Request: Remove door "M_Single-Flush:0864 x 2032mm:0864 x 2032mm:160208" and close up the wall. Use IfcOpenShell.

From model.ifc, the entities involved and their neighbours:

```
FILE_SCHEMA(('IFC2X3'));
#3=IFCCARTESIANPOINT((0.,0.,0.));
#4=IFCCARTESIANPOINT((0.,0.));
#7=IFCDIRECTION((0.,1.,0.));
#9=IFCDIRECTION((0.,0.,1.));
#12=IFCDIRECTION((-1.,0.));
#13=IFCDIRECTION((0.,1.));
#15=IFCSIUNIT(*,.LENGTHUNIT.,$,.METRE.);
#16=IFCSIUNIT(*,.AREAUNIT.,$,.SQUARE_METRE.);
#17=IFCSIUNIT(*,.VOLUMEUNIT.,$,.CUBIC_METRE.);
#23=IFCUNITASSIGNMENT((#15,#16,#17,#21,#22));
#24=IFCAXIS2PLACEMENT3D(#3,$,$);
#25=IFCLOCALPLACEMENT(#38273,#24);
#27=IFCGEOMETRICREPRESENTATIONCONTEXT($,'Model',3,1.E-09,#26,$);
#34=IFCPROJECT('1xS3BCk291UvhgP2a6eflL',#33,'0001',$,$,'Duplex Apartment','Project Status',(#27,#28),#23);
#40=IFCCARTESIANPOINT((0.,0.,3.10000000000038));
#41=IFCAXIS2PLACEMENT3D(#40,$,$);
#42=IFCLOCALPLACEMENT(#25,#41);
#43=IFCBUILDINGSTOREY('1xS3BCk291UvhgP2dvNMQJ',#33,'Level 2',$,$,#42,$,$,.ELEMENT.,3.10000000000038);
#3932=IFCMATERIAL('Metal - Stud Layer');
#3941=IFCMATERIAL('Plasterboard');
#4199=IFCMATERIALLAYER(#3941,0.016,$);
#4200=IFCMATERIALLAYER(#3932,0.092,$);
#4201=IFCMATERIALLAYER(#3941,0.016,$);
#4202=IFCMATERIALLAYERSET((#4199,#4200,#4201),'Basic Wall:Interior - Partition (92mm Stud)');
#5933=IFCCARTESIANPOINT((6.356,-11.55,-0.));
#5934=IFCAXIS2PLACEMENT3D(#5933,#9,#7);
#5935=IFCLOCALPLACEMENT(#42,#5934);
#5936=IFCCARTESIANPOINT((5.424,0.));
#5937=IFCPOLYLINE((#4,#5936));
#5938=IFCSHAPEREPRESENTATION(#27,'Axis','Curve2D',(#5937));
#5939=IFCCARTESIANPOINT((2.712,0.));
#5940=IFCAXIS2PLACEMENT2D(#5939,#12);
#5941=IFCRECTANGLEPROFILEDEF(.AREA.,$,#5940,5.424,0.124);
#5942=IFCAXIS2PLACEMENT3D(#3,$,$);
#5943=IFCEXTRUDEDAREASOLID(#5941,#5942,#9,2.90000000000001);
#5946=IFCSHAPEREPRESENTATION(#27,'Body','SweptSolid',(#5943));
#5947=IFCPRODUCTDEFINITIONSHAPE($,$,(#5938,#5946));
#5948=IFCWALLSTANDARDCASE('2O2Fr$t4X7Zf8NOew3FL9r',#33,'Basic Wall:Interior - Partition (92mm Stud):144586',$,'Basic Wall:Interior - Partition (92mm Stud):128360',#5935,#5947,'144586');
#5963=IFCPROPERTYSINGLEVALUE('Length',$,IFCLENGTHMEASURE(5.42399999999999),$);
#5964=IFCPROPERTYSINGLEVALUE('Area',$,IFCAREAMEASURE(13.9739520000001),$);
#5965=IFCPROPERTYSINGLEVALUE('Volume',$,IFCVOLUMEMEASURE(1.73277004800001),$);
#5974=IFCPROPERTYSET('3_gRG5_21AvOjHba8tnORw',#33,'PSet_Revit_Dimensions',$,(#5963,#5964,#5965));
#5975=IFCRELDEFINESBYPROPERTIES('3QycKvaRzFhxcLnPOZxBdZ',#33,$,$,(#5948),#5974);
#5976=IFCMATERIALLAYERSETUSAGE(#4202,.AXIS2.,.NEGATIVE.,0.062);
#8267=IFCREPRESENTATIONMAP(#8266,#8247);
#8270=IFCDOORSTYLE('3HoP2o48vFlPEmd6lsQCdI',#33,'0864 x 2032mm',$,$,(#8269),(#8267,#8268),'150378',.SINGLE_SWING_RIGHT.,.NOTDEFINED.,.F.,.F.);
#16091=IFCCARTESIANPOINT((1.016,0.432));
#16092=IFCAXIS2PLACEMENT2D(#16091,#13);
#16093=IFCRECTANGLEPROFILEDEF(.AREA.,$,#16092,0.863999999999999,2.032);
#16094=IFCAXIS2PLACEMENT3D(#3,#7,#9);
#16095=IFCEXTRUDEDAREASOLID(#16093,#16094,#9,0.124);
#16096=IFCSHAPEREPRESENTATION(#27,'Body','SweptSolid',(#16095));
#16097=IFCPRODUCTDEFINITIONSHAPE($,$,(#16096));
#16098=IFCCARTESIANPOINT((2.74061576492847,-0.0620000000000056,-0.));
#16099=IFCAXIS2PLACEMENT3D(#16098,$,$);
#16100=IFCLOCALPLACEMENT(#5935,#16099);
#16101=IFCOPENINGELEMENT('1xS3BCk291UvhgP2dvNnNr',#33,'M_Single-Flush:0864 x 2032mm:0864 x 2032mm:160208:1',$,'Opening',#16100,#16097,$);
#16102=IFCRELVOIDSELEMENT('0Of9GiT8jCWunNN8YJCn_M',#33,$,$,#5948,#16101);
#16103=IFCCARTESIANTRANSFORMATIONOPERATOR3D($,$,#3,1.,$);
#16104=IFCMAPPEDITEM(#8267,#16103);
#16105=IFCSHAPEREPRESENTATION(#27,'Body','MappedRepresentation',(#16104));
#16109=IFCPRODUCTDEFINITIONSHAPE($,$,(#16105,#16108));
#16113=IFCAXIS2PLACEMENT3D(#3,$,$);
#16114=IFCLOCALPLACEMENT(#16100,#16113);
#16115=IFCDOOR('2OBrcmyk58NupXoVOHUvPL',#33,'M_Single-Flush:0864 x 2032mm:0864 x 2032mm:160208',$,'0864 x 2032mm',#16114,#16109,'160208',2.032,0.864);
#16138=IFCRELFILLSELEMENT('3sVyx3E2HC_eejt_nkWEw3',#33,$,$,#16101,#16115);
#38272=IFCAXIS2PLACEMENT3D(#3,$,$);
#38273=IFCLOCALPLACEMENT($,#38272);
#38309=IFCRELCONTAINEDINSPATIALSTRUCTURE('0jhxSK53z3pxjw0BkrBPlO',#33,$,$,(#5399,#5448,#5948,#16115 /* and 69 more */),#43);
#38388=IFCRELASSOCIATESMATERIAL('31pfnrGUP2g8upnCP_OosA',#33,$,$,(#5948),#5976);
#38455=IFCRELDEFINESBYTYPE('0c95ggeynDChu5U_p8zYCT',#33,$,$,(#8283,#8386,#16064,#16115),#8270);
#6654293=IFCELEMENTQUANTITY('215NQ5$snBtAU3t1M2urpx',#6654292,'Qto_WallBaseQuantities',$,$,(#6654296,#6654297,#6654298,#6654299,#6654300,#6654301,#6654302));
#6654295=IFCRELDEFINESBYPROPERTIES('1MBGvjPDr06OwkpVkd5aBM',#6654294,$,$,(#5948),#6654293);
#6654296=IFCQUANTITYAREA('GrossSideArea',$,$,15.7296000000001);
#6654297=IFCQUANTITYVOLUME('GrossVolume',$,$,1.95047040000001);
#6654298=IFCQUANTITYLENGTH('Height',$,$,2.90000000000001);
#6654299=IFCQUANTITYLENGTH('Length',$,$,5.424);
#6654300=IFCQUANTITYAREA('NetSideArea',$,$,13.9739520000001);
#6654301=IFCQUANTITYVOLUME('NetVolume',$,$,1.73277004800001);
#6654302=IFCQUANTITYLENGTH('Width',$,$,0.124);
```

```python
import ifcopenshell
import ifcopenshell.api.feature
import ifcopenshell.api.pset
import ifcopenshell.api.root
import ifcopenshell.geom
import ifcopenshell.util.element
import ifcopenshell.util.shape
import ifcopenshell.util.unit

model = ifcopenshell.open("model.ifc")
area_scale = ifcopenshell.util.unit.calculate_unit_scale(model, "AREAUNIT")
volume_scale = ifcopenshell.util.unit.calculate_unit_scale(model, "VOLUMEUNIT")
settings = ifcopenshell.geom.settings()


def volume(element):
    """Net volume in cubic metres, openings subtracted."""
    shape = ifcopenshell.geom.create_shape(settings, element)
    return ifcopenshell.util.shape.get_volume(shape.geometry)


door = model.by_guid("2OBrcmyk58NupXoVOHUvPL")
opening = door.FillsVoids[0].RelatingOpeningElement
wall = opening.VoidsElements[0].RelatingBuildingElement
before = volume(wall)

ifcopenshell.api.root.remove_product(model, product=door)
ifcopenshell.api.feature.remove_feature(model, feature=opening)

after = volume(wall)
thickness = 0.124  # wall thickness in metres

# Update the wall's stored quantities.
pset = model.by_id(ifcopenshell.util.element.get_pset(wall, "PSet_Revit_Dimensions", should_inherit=False)["id"])
ifcopenshell.api.pset.edit_pset(model, pset=pset, properties={
    "Area": model.create_entity("IfcAreaMeasure", after / thickness / area_scale),
    "Volume": model.create_entity("IfcVolumeMeasure", after / volume_scale),
})
qto = model.by_id(ifcopenshell.util.element.get_pset(wall, "Qto_WallBaseQuantities", should_inherit=False)["id"])
ifcopenshell.api.pset.edit_qto(model, qto=qto, properties={
    "NetSideArea": after / thickness / area_scale,
    "NetVolume": after / volume_scale,
})

print(f"wall volume {before:.3f} -> {after:.3f} m3")

model.write("model_v2.ifc")
```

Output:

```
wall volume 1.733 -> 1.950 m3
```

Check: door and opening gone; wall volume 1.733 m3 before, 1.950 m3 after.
